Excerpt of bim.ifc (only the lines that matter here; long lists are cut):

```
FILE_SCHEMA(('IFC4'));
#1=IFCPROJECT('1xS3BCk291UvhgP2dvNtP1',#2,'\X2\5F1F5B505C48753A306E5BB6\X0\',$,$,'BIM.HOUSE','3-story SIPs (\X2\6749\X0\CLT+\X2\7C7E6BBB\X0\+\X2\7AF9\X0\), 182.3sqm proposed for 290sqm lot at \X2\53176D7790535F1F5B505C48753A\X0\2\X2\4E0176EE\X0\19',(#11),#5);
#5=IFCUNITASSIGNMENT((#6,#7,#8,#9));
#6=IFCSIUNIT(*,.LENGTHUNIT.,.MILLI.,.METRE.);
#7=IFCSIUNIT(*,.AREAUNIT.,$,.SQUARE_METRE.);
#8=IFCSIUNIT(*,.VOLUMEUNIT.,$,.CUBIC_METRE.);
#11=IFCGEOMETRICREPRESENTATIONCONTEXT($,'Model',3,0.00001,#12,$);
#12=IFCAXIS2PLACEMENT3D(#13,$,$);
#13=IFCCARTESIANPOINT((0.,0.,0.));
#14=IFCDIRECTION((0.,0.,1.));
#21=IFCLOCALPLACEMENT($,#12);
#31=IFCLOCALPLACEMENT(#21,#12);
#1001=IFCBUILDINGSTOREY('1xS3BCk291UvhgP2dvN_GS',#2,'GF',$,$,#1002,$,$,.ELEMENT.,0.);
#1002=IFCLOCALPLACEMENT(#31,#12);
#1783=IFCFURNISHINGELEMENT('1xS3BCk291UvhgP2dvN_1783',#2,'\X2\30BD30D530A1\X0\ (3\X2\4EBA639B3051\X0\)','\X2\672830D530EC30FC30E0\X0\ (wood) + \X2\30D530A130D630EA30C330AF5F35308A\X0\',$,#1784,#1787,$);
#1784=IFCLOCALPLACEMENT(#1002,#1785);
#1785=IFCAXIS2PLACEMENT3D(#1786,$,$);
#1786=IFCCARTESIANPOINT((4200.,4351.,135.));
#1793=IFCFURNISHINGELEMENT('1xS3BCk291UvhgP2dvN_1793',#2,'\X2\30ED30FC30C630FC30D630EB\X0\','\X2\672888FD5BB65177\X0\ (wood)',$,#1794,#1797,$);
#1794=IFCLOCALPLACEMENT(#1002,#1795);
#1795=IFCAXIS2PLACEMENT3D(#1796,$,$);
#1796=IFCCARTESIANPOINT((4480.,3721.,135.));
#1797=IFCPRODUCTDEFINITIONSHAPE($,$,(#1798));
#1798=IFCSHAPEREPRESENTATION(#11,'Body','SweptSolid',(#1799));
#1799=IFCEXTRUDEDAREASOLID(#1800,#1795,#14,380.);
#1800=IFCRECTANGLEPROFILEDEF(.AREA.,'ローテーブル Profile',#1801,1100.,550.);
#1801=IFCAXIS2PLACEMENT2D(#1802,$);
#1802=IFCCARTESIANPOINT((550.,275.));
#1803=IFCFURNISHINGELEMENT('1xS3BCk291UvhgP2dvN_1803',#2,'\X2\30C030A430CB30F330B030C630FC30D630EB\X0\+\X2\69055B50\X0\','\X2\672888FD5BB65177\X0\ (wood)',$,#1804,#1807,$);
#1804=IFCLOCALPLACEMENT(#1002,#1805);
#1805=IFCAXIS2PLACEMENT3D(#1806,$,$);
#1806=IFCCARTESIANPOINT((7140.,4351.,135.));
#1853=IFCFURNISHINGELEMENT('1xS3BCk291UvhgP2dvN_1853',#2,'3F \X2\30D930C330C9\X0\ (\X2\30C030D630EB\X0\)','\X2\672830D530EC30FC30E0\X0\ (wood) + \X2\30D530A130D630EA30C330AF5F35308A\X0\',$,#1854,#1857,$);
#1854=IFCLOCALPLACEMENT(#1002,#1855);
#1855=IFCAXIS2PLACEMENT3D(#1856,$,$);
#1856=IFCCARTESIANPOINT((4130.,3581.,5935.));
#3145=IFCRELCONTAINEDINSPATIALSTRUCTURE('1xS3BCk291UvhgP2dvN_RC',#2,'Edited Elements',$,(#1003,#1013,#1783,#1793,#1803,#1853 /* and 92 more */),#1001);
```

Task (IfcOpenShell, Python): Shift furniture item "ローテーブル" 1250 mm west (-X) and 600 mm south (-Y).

```python
import ifcopenshell
import ifcopenshell.api.geometry
import ifcopenshell.util.placement

model = ifcopenshell.open("bim.ifc")

item = model.by_guid("1xS3BCk291UvhgP2dvN_1793")
matrix = ifcopenshell.util.placement.get_local_placement(item.ObjectPlacement)
matrix[0, 3] -= 1250.0
matrix[1, 3] -= 600.0
ifcopenshell.api.geometry.edit_object_placement(model, product=item, matrix=matrix, is_si=False)

print(ifcopenshell.util.placement.get_local_placement(item.ObjectPlacement).round(3) + 0.0)

model.write("bim_v2.ifc")
```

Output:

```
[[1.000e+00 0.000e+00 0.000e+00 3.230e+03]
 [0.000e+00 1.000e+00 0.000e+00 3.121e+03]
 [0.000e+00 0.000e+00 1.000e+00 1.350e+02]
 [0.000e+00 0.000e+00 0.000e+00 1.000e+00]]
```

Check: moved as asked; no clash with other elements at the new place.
